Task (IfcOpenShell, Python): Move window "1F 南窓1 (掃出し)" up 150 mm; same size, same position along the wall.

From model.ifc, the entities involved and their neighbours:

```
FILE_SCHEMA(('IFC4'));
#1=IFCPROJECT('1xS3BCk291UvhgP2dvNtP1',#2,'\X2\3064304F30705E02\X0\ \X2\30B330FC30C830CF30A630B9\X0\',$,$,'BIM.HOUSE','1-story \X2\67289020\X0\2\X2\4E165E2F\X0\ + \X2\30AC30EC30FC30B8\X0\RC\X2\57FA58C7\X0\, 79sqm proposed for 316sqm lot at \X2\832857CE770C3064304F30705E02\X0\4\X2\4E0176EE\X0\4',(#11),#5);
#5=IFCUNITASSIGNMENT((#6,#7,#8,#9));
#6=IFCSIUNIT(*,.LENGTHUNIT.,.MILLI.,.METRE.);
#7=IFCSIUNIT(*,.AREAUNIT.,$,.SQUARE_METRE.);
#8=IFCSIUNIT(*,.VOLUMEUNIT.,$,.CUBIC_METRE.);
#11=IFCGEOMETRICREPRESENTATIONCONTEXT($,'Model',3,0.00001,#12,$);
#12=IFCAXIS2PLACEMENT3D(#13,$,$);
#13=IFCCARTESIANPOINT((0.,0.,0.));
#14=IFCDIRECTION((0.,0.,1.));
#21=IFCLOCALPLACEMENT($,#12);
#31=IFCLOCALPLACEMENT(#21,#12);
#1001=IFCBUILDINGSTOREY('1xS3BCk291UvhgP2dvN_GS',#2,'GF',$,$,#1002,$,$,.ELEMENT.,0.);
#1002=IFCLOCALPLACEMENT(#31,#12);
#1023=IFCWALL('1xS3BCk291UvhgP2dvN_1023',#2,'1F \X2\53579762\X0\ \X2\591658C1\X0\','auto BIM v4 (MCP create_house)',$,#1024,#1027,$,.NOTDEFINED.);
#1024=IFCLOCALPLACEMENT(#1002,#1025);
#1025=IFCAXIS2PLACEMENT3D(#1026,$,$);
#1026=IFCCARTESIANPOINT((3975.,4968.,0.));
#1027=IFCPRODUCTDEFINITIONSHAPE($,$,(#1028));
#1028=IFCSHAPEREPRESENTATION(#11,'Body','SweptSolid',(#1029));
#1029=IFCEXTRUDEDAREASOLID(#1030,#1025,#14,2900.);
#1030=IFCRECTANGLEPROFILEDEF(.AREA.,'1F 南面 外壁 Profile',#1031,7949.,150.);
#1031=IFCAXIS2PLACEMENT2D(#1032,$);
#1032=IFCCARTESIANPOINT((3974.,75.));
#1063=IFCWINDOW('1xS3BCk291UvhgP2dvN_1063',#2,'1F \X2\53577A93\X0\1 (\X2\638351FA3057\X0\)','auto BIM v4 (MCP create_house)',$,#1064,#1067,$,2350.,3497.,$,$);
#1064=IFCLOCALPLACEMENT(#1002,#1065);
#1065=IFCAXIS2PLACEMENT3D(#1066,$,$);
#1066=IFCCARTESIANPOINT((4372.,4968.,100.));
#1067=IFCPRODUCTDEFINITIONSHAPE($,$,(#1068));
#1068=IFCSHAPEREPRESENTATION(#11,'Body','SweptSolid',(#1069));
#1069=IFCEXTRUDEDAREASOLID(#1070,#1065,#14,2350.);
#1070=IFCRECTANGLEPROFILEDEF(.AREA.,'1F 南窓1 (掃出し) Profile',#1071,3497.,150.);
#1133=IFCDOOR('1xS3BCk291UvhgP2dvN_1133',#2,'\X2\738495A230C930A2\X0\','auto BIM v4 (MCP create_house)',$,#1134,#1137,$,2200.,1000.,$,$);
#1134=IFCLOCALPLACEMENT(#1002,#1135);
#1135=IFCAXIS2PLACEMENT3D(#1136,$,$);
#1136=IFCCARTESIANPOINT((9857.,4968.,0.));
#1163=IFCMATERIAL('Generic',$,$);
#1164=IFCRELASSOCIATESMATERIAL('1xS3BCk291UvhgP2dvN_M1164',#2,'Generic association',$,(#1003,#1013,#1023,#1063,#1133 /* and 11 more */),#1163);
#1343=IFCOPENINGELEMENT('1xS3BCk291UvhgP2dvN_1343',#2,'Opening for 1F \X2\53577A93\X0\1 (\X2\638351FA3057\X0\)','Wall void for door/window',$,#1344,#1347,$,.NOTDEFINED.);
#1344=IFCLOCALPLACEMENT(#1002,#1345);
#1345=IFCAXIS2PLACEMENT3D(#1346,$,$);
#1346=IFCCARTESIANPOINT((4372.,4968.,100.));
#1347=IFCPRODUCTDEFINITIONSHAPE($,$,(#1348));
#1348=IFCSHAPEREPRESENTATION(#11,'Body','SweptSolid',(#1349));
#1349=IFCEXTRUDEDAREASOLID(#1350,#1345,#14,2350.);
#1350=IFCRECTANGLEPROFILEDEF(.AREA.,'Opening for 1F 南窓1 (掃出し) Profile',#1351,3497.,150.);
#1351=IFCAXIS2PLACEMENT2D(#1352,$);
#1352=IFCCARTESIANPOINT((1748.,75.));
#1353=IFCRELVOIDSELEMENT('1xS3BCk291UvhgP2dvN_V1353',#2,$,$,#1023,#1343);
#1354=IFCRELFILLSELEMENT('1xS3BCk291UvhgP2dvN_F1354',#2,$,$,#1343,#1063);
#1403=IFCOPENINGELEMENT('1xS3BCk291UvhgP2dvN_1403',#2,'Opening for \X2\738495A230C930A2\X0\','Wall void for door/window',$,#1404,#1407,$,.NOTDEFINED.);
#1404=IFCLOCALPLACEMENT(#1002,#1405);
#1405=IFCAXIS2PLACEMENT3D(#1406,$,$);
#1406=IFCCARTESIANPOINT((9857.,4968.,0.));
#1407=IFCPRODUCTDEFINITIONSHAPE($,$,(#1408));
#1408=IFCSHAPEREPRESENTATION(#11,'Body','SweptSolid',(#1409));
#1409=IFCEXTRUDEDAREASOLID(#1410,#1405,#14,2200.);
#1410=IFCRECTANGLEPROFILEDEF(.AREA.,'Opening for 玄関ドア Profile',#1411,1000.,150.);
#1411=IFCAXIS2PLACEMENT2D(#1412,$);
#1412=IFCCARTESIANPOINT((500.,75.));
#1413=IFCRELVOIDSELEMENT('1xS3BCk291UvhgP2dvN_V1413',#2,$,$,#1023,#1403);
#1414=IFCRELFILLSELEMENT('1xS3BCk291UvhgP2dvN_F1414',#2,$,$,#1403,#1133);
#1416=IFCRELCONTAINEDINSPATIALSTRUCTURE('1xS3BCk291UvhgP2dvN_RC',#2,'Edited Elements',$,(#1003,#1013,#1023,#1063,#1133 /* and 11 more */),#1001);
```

```python
import numpy as np
import ifcopenshell
import ifcopenshell.api.geometry
import ifcopenshell.util.placement
import ifcopenshell.util.unit

model = ifcopenshell.open("model.ifc")
unit_scale = ifcopenshell.util.unit.calculate_unit_scale(model)

window = model.by_guid("1xS3BCk291UvhgP2dvN_1063")
opening = window.FillsVoids[0].RelatingOpeningElement
dz = 0.15 / unit_scale

shift = np.array([0.0, 0.0, dz])
# The window is not placed relative to its opening, so move both.
for product in (opening, window):
    matrix = ifcopenshell.util.placement.get_local_placement(product.ObjectPlacement)
    matrix[:3, 3] += shift
    ifcopenshell.api.geometry.edit_object_placement(model, product=product, matrix=matrix, is_si=False)

print(f"moved by {dz * unit_scale:+.3f} m")

model.write("model_rev.ifc")
```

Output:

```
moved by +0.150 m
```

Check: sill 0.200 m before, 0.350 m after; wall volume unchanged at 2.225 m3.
